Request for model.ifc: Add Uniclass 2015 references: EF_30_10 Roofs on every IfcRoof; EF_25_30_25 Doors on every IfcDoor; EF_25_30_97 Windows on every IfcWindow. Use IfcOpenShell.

First a look at what the model holds.

```python
import ifcopenshell

model = ifcopenshell.open("model.ifc")
print(model.schema)
print("classifications:", [c.Name for c in model.by_type("IfcClassification")])
for ifc_class in ("IfcDoor", "IfcRoof", "IfcStair", "IfcWall", "IfcWindow"):
    print(ifc_class, len(model.by_type(ifc_class)))
```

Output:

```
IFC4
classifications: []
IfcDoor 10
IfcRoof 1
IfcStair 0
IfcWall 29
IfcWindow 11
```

```python
import ifcopenshell
import ifcopenshell.api.classification

model = ifcopenshell.open("model.ifc")

system = ifcopenshell.api.classification.add_classification(model, classification="Uniclass 2015")

codes = {
    "IfcRoof": ("EF_30_10", "Roofs"),
    "IfcDoor": ("EF_25_30_25", "Doors"),
    "IfcWindow": ("EF_25_30_97", "Windows"),
}
for ifc_class, (code, name) in codes.items():
    products = model.by_type(ifc_class)
    ifcopenshell.api.classification.add_reference(
        model, products=products, classification=system, identification=code, name=name
    )
    print(code, len(products))

model.write("model_updated.ifc")
```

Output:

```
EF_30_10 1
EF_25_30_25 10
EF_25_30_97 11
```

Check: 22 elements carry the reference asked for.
